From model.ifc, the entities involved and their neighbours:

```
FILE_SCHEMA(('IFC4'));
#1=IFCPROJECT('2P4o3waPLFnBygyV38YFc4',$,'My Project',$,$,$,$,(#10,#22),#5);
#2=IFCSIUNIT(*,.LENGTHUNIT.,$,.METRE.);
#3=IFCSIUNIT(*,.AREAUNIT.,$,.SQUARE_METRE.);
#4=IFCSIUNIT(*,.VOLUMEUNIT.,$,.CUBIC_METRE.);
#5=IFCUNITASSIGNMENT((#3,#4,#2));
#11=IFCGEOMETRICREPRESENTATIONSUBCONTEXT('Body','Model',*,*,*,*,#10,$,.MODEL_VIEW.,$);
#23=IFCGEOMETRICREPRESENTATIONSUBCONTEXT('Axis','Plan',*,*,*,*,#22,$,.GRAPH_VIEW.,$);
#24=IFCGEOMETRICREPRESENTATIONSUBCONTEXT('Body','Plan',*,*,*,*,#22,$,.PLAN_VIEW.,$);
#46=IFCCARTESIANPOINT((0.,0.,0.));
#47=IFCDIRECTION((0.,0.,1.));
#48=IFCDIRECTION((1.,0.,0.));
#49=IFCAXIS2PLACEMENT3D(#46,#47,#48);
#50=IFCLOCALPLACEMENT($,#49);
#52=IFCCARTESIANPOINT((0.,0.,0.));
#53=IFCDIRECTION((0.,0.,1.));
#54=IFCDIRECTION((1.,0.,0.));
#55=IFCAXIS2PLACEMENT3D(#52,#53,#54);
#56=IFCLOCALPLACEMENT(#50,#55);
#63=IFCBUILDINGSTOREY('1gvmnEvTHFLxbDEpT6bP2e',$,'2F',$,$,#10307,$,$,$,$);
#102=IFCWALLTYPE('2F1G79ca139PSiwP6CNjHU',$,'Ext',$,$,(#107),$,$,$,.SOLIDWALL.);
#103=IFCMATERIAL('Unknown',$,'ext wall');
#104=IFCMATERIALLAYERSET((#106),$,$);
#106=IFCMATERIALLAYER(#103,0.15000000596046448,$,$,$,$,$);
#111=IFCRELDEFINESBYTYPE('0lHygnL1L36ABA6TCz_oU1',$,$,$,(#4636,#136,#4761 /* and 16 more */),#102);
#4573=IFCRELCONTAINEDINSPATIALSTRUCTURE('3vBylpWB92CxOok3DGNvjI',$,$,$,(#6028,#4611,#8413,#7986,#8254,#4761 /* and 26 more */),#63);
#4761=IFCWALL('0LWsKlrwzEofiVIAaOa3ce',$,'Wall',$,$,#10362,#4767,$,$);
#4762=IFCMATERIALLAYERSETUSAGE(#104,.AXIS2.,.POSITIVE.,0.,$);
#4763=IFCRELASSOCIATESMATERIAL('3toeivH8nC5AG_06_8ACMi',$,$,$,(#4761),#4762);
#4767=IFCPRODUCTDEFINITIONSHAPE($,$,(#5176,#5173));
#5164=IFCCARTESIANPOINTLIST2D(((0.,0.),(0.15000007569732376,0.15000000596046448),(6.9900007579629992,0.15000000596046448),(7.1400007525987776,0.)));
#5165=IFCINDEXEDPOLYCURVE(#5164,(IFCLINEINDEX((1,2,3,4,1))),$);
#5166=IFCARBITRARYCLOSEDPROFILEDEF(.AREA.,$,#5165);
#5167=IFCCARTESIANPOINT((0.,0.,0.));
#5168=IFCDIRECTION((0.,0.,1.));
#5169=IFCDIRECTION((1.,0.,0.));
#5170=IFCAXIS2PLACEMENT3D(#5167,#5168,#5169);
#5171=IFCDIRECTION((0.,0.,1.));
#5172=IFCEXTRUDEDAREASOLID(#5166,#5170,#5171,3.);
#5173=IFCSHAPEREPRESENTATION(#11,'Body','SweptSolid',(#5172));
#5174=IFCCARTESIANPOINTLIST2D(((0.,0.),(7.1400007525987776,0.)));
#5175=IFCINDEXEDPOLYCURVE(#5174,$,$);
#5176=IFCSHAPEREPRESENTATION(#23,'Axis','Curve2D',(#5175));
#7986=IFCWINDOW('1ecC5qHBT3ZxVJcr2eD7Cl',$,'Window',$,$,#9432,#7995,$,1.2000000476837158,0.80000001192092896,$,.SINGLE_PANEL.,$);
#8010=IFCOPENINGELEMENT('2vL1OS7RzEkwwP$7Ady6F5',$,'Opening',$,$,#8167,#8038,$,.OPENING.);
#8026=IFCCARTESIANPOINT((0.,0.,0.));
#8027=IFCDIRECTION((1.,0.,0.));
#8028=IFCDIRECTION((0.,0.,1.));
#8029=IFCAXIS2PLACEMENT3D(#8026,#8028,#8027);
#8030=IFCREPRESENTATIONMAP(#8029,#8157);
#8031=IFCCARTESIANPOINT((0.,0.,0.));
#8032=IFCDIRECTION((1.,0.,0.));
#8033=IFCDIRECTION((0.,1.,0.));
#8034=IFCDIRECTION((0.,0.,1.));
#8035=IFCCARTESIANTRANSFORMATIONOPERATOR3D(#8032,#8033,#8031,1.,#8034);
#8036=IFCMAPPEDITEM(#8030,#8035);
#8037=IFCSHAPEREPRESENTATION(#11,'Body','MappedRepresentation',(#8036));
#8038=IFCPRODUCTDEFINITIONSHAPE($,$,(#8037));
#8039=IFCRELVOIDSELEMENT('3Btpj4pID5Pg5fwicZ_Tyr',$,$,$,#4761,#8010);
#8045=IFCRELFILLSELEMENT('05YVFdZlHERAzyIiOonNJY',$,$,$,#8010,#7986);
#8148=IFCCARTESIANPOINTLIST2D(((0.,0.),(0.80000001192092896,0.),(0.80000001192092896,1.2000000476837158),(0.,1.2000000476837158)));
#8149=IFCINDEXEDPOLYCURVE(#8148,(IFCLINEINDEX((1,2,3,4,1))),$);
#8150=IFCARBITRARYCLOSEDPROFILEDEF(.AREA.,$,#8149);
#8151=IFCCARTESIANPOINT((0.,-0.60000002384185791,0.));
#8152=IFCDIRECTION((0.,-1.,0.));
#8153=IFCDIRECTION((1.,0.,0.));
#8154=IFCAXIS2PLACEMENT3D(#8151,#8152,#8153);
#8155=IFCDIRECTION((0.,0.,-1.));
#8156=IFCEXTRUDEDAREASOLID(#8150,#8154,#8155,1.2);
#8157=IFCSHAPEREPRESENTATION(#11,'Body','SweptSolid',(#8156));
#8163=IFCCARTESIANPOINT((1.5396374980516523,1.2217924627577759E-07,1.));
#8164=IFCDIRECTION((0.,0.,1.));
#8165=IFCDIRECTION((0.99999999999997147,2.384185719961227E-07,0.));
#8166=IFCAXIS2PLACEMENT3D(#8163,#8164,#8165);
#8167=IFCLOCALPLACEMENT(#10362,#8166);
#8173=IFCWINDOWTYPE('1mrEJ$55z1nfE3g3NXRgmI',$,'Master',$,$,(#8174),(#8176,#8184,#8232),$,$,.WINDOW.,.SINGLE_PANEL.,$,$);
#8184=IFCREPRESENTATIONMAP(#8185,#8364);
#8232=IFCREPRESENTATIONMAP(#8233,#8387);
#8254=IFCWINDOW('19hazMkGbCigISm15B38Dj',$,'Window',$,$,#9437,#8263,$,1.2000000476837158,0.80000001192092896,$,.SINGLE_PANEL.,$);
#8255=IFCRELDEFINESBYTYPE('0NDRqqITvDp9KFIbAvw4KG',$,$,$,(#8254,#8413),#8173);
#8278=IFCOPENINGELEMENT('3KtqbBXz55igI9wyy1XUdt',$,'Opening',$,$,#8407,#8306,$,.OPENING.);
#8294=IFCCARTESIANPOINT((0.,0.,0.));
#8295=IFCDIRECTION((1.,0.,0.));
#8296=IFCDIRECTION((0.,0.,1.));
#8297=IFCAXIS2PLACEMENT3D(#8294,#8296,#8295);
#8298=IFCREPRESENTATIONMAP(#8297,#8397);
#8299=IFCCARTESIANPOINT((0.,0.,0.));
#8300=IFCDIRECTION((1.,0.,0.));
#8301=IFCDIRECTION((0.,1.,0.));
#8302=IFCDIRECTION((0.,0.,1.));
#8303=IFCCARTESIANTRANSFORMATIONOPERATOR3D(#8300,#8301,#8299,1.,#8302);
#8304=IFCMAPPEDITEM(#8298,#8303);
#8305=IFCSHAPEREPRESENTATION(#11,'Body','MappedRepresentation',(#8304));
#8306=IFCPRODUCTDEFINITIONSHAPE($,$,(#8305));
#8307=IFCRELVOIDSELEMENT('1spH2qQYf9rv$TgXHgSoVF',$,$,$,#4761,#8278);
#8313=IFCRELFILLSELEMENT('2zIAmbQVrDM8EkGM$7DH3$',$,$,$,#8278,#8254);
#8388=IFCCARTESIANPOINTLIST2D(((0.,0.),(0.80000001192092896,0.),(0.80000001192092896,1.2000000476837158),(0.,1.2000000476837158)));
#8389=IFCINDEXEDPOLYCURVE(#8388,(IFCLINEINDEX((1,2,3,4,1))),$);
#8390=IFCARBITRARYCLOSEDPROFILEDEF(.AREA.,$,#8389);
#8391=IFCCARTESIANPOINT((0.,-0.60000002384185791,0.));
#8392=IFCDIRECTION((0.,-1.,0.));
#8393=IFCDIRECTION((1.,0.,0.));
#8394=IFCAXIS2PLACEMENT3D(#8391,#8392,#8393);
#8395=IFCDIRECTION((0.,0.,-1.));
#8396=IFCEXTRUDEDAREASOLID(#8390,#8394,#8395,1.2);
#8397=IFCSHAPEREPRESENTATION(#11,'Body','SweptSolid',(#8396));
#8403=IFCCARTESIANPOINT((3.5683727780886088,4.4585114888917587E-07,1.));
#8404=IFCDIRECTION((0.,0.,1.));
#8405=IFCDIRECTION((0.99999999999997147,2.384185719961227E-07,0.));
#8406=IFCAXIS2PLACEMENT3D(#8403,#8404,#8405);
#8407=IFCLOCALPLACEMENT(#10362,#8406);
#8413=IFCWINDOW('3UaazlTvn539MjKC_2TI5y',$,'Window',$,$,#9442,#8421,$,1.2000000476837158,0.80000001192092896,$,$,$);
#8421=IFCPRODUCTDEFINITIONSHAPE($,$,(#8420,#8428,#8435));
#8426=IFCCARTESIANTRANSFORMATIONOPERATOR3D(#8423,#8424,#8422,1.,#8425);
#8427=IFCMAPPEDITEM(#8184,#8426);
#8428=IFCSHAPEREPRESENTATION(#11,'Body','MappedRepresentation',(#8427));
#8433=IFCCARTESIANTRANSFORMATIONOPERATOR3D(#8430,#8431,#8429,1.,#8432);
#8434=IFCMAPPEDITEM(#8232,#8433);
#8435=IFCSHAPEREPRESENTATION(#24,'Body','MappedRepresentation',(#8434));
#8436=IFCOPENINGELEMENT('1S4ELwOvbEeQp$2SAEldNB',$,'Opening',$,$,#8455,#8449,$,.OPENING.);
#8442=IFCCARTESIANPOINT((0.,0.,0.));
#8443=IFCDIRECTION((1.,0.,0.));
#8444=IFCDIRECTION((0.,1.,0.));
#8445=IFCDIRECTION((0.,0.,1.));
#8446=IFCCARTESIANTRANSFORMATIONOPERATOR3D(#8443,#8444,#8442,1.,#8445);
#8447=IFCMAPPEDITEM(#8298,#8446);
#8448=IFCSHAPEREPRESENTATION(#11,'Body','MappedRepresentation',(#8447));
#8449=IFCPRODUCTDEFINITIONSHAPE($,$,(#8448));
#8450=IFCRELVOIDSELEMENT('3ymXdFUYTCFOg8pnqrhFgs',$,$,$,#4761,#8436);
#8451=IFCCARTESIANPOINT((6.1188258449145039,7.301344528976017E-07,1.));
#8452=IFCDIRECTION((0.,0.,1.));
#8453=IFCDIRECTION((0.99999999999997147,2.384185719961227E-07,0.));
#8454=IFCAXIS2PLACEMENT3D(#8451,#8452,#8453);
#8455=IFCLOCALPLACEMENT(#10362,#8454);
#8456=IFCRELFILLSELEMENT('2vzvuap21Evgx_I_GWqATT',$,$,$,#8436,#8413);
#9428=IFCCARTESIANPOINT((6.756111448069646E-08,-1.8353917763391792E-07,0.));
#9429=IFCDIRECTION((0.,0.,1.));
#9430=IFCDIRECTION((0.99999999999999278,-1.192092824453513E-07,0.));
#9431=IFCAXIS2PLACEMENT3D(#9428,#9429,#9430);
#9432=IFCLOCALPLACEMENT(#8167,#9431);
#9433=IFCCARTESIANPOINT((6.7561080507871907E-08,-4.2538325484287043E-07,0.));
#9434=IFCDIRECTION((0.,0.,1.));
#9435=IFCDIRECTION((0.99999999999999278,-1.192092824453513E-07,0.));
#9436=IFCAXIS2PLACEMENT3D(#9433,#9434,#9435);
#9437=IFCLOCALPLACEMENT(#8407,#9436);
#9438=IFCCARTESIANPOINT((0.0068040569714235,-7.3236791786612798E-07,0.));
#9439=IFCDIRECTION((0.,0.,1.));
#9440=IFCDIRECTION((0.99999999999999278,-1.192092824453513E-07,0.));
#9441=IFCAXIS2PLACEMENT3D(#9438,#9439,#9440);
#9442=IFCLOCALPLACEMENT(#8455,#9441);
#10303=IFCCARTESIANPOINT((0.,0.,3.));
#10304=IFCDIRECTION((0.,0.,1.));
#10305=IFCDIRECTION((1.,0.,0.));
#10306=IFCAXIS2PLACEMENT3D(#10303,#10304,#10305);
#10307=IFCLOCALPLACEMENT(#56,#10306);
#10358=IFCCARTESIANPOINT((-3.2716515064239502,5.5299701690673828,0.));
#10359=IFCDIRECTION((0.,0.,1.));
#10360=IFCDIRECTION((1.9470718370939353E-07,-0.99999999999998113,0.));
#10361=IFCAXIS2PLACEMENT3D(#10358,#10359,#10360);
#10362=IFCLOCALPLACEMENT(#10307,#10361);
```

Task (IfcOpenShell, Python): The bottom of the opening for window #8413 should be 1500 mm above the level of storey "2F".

```python
import numpy as np
import ifcopenshell
import ifcopenshell.api.geometry
import ifcopenshell.geom
import ifcopenshell.util.element
import ifcopenshell.util.placement
import ifcopenshell.util.shape
import ifcopenshell.util.unit

model = ifcopenshell.open("model.ifc")
unit_scale = ifcopenshell.util.unit.calculate_unit_scale(model)

window = model.by_guid("3UaazlTvn539MjKC_2TI5y")
opening = window.FillsVoids[0].RelatingOpeningElement
storey = ifcopenshell.util.element.get_container(window, ifc_class="IfcBuildingStorey")
level = ifcopenshell.util.placement.get_local_placement(storey.ObjectPlacement)[2, 3]

# The opening's origin need not be at the sill, so measure its lowest point.
shape = ifcopenshell.geom.create_shape(ifcopenshell.geom.settings(), opening)
bottom = ifcopenshell.util.shape.get_shape_bottom_elevation(shape, shape.geometry) / unit_scale
dz = level + 1.5 / unit_scale - bottom

shift = np.array([0.0, 0.0, dz])
# The window is placed relative to its opening, so it follows when the opening moves.
matrix = ifcopenshell.util.placement.get_local_placement(opening.ObjectPlacement)
matrix[:3, 3] += shift
ifcopenshell.api.geometry.edit_object_placement(
    model, product=opening, matrix=matrix, is_si=False, should_transform_children=True
)

print(f"moved by {dz * unit_scale:+.3f} m")

model.write("model_updated.ifc")
```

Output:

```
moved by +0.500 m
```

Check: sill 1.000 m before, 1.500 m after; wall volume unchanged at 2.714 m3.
